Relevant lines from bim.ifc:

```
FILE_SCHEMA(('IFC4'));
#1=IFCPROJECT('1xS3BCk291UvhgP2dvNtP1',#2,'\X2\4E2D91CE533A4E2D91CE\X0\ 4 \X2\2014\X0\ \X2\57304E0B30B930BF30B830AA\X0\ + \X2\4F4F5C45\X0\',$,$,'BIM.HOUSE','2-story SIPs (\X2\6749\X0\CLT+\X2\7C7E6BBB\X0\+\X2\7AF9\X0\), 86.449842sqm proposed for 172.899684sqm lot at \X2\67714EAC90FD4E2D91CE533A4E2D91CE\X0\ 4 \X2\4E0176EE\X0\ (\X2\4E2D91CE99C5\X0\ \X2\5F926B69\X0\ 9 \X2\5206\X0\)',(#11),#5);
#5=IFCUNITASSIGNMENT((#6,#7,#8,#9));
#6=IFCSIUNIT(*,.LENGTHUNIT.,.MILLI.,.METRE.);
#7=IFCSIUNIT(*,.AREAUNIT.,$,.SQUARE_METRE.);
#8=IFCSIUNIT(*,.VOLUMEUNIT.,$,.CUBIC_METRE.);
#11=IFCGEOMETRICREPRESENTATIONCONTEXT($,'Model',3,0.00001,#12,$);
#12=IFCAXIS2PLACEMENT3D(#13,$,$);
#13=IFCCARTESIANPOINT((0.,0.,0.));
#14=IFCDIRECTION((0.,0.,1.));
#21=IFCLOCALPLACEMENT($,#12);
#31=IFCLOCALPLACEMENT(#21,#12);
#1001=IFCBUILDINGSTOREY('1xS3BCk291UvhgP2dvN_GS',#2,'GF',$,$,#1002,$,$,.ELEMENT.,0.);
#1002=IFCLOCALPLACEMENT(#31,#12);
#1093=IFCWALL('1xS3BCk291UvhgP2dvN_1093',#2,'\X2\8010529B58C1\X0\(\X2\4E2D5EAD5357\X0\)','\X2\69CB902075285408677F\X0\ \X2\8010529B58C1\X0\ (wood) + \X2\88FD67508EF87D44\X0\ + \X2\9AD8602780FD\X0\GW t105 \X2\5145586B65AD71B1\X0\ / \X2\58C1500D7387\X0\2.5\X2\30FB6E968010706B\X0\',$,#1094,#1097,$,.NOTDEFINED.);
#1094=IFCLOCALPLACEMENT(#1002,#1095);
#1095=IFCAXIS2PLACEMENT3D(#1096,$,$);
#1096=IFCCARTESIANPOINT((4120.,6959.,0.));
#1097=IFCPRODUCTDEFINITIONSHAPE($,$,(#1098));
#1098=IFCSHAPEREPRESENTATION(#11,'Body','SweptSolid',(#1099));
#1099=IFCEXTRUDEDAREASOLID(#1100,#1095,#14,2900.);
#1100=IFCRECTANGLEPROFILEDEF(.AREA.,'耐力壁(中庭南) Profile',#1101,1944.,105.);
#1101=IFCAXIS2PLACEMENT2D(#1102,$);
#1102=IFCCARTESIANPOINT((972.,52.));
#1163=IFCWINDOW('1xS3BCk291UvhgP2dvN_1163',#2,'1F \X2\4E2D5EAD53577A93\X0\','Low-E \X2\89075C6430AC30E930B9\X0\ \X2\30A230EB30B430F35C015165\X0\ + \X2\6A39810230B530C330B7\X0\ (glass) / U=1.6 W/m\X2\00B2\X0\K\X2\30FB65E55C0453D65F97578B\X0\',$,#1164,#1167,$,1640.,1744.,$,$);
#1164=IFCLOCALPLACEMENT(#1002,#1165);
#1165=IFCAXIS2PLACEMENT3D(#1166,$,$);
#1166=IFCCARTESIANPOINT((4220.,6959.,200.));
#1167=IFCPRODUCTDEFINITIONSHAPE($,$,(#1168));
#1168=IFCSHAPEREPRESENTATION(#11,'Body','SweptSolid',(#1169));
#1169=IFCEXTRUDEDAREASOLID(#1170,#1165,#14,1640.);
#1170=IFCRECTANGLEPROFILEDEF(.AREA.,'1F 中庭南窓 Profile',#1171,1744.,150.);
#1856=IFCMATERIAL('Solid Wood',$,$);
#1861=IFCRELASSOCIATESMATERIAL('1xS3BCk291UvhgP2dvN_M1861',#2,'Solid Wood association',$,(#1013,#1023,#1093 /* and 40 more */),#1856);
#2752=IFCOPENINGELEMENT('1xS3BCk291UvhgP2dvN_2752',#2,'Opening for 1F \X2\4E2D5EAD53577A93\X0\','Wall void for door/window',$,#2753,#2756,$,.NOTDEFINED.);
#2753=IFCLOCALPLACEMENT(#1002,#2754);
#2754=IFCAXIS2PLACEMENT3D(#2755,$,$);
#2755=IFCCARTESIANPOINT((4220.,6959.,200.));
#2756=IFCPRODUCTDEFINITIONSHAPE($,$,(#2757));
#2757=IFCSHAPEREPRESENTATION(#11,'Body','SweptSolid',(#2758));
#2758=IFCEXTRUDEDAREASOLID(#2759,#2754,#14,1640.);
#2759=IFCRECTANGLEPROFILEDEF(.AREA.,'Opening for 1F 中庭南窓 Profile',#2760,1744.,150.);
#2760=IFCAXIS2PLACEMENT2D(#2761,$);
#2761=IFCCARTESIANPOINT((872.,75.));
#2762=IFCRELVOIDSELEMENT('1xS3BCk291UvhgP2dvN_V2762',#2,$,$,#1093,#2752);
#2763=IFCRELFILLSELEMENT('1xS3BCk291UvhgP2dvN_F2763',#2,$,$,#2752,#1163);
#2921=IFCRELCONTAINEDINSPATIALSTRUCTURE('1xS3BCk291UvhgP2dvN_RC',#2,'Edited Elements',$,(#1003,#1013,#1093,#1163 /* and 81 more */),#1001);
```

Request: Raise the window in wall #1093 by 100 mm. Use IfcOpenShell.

```python
import numpy as np
import ifcopenshell
import ifcopenshell.api.geometry
import ifcopenshell.util.placement
import ifcopenshell.util.unit

model = ifcopenshell.open("bim.ifc")
unit_scale = ifcopenshell.util.unit.calculate_unit_scale(model)

window = model.by_id(1163)
opening = window.FillsVoids[0].RelatingOpeningElement
dz = 100.0

shift = np.array([0.0, 0.0, dz])
# The window is not placed relative to its opening, so move both.
for product in (opening, window):
    matrix = ifcopenshell.util.placement.get_local_placement(product.ObjectPlacement)
    matrix[:3, 3] += shift
    ifcopenshell.api.geometry.edit_object_placement(model, product=product, matrix=matrix, is_si=False)

print(f"moved by {dz * unit_scale:+.3f} m")

model.write("bim_rev.ifc")
```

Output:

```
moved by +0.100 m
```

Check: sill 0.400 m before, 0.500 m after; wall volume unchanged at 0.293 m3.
